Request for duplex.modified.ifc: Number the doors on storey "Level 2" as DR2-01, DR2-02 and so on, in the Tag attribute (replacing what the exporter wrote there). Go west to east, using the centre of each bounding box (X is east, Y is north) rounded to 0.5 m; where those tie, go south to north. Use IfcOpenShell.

First a look at what the model holds.

```python
import ifcopenshell
import ifcopenshell.util.element
import ifcopenshell.util.placement

model = ifcopenshell.open("duplex.modified.ifc")
print(model.schema)
storey = next(s for s in model.by_type("IfcBuildingStorey") if s.Name == "Level 2")
doors = [e for e in ifcopenshell.util.element.get_decomposition(storey) if e.is_a("IfcDoor")]
for e in sorted(doors, key=lambda e: e.id()):
    origin = ifcopenshell.util.placement.get_local_placement(e.ObjectPlacement)[:3, 3]
    print(e.id(), e.Tag, e.Name, origin.round(2) + 0.0, sep=" | ")
```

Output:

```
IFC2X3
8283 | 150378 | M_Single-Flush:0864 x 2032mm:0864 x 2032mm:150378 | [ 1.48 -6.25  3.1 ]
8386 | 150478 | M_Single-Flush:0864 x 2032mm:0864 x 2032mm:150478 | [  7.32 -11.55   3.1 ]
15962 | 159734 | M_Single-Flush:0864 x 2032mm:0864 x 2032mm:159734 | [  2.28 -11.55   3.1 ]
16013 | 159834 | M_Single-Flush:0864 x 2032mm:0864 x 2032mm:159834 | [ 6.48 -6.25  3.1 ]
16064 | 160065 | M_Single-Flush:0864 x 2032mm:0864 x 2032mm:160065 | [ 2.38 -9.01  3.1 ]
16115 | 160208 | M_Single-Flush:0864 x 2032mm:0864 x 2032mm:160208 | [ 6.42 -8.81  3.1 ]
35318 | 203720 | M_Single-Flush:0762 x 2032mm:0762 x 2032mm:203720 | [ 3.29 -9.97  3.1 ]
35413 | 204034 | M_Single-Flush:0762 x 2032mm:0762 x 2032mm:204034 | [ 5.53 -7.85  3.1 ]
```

```python
import ifcopenshell
import ifcopenshell.geom
import ifcopenshell.util.element
import ifcopenshell.util.shape

model = ifcopenshell.open("duplex.modified.ifc")
settings = ifcopenshell.geom.settings()
settings.set("use-world-coords", True)


def centre(element):
    shape = ifcopenshell.geom.create_shape(settings, element)
    return ifcopenshell.util.shape.get_bbox_centroid(shape.geometry)


storey = next(s for s in model.by_type("IfcBuildingStorey") if s.Name == "Level 2")
doors = [e for e in ifcopenshell.util.element.get_decomposition(storey) if e.is_a("IfcDoor")]

# Insertion points can sit at a corner or the storey origin, so sort by the geometry (in metres).
centres = {e: centre(e) for e in doors}
doors.sort(key=lambda e: (round(centres[e][0] / 0.5), centres[e][1]))

for i, e in enumerate(doors, start=1):
    number = f"DR2-{i:02d}"
    e.Tag = number
    print(e.id(), number)

model.write("duplex.modified_v2.ifc")
```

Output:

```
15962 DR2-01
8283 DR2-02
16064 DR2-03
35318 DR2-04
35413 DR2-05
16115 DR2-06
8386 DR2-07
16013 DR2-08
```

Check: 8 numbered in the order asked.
